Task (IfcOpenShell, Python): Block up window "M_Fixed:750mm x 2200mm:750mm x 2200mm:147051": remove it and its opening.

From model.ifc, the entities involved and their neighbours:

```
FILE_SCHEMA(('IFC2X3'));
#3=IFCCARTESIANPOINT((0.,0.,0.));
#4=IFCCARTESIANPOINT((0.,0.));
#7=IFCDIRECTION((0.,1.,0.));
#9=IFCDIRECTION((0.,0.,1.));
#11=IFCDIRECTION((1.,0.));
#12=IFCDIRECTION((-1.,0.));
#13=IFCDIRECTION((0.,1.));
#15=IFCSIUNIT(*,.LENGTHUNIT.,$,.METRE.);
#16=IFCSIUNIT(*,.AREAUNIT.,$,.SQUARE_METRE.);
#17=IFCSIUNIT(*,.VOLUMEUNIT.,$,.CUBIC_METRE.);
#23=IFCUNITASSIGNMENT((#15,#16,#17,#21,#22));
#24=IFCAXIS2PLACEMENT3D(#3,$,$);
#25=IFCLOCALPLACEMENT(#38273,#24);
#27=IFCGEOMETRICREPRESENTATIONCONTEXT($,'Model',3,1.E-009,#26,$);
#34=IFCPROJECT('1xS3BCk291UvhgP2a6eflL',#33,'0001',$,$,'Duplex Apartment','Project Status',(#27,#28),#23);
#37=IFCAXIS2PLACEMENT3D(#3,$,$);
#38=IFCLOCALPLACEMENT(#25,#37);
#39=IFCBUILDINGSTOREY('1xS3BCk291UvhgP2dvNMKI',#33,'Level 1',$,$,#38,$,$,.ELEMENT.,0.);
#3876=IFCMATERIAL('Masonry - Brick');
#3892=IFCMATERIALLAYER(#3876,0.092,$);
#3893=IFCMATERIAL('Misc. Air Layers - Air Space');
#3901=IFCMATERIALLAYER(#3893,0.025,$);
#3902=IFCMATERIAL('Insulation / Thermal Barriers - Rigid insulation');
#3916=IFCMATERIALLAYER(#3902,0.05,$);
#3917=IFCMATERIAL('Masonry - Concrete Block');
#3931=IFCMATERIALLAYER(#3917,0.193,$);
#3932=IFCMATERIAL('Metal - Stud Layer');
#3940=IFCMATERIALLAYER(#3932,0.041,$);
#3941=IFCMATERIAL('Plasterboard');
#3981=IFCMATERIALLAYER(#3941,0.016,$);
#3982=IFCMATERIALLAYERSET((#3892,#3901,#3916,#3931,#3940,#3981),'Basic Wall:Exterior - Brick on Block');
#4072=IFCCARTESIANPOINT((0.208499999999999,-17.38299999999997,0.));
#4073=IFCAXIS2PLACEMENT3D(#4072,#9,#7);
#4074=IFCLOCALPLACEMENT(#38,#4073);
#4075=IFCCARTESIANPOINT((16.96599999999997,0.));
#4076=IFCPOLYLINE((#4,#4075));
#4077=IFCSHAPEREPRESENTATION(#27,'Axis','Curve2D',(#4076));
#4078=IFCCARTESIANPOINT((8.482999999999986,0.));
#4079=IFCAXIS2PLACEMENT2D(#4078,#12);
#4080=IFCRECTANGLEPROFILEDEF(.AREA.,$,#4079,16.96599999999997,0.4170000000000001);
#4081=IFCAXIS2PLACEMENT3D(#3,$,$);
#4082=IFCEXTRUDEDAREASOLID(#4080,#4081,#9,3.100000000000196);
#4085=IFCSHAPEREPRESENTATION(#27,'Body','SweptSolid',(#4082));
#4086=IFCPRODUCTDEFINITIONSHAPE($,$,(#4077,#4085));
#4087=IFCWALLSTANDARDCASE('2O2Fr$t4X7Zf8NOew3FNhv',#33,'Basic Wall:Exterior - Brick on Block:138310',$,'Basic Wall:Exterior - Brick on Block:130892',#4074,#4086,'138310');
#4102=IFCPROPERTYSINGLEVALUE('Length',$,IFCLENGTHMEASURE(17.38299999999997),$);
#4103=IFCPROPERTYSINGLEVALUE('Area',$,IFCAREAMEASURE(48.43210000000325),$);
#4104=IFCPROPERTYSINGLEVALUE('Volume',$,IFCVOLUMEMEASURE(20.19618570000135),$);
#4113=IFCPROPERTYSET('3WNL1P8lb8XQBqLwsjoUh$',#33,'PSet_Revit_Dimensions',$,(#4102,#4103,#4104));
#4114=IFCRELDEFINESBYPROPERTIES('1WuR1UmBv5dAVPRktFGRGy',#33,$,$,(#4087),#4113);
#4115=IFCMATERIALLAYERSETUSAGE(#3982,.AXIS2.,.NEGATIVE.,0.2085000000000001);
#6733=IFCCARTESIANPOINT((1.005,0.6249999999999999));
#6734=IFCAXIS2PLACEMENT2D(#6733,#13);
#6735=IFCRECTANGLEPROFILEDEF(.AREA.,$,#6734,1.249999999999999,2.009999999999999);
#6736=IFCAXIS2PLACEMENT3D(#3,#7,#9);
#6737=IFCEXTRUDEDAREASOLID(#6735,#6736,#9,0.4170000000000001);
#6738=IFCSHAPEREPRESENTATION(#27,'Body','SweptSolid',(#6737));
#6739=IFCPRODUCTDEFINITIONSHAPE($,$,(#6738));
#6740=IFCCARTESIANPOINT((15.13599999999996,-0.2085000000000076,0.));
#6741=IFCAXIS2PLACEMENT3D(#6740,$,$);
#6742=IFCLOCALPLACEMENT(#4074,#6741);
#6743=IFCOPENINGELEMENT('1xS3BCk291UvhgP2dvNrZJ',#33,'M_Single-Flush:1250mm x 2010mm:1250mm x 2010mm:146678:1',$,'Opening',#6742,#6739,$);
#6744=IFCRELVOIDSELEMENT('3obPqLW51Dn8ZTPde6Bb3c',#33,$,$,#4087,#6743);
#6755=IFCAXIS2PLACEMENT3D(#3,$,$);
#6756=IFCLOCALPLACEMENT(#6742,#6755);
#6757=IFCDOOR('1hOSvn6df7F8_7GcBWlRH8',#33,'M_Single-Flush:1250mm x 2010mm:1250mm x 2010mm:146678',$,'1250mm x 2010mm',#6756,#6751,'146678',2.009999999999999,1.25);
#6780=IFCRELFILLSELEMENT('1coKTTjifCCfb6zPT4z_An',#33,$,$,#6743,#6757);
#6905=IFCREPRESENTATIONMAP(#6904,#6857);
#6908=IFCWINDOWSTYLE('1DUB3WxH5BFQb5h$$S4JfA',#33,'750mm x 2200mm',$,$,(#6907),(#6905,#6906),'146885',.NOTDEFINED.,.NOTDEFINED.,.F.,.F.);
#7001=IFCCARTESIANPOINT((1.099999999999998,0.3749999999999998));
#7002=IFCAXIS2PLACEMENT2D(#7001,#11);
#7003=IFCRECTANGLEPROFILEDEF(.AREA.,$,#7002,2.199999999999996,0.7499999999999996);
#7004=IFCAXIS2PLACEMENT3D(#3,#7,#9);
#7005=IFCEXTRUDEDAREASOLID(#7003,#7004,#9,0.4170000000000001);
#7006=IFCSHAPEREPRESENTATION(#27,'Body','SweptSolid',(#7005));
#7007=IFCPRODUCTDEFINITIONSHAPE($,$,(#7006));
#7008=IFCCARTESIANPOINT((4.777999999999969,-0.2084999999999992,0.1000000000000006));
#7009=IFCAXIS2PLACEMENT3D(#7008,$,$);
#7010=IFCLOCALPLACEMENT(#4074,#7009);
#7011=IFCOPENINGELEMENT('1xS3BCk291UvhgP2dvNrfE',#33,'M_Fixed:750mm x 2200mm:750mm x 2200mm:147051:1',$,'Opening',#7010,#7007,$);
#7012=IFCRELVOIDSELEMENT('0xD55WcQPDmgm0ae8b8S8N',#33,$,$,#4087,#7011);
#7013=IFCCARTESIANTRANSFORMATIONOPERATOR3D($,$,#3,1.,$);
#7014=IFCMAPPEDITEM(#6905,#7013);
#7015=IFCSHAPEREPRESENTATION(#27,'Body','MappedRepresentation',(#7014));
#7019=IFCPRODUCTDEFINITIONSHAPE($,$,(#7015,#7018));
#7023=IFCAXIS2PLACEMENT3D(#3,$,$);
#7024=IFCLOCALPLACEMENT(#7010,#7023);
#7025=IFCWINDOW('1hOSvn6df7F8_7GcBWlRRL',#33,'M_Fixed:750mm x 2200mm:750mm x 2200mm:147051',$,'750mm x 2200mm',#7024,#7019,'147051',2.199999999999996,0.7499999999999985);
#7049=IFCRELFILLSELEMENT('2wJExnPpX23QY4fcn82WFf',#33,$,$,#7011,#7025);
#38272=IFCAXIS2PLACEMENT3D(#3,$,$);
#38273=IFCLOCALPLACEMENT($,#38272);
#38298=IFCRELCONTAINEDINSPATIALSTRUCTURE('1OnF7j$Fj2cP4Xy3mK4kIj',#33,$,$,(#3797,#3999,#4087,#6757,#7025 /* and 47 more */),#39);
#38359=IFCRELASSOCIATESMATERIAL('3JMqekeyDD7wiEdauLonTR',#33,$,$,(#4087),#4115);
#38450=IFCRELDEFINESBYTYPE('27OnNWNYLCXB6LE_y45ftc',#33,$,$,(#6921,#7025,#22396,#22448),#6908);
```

```python
import ifcopenshell
import ifcopenshell.api.feature
import ifcopenshell.api.pset
import ifcopenshell.api.root
import ifcopenshell.geom
import ifcopenshell.util.element
import ifcopenshell.util.shape
import ifcopenshell.util.unit

model = ifcopenshell.open("model.ifc")
area_scale = ifcopenshell.util.unit.calculate_unit_scale(model, "AREAUNIT")
volume_scale = ifcopenshell.util.unit.calculate_unit_scale(model, "VOLUMEUNIT")
settings = ifcopenshell.geom.settings()


def volume(element):
    """Net volume in cubic metres, openings subtracted."""
    shape = ifcopenshell.geom.create_shape(settings, element)
    return ifcopenshell.util.shape.get_volume(shape.geometry)


window = model.by_id(7025)
opening = window.FillsVoids[0].RelatingOpeningElement
wall = opening.VoidsElements[0].RelatingBuildingElement
before = volume(wall)

ifcopenshell.api.root.remove_product(model, product=window)
ifcopenshell.api.feature.remove_feature(model, feature=opening)

after = volume(wall)
thickness = 0.417  # wall thickness in metres

# Update the wall's stored quantities.
pset = model.by_id(ifcopenshell.util.element.get_pset(wall, "PSet_Revit_Dimensions", should_inherit=False)["id"])
ifcopenshell.api.pset.edit_pset(model, pset=pset, properties={
    "Area": model.create_entity("IfcAreaMeasure", after / thickness / area_scale),
    "Volume": model.create_entity("IfcVolumeMeasure", after / volume_scale),
})

print(f"wall volume {before:.3f} -> {after:.3f} m3")

model.write("model_v2.ifc")
```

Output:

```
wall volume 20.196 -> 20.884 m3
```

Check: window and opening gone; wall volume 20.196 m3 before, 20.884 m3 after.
